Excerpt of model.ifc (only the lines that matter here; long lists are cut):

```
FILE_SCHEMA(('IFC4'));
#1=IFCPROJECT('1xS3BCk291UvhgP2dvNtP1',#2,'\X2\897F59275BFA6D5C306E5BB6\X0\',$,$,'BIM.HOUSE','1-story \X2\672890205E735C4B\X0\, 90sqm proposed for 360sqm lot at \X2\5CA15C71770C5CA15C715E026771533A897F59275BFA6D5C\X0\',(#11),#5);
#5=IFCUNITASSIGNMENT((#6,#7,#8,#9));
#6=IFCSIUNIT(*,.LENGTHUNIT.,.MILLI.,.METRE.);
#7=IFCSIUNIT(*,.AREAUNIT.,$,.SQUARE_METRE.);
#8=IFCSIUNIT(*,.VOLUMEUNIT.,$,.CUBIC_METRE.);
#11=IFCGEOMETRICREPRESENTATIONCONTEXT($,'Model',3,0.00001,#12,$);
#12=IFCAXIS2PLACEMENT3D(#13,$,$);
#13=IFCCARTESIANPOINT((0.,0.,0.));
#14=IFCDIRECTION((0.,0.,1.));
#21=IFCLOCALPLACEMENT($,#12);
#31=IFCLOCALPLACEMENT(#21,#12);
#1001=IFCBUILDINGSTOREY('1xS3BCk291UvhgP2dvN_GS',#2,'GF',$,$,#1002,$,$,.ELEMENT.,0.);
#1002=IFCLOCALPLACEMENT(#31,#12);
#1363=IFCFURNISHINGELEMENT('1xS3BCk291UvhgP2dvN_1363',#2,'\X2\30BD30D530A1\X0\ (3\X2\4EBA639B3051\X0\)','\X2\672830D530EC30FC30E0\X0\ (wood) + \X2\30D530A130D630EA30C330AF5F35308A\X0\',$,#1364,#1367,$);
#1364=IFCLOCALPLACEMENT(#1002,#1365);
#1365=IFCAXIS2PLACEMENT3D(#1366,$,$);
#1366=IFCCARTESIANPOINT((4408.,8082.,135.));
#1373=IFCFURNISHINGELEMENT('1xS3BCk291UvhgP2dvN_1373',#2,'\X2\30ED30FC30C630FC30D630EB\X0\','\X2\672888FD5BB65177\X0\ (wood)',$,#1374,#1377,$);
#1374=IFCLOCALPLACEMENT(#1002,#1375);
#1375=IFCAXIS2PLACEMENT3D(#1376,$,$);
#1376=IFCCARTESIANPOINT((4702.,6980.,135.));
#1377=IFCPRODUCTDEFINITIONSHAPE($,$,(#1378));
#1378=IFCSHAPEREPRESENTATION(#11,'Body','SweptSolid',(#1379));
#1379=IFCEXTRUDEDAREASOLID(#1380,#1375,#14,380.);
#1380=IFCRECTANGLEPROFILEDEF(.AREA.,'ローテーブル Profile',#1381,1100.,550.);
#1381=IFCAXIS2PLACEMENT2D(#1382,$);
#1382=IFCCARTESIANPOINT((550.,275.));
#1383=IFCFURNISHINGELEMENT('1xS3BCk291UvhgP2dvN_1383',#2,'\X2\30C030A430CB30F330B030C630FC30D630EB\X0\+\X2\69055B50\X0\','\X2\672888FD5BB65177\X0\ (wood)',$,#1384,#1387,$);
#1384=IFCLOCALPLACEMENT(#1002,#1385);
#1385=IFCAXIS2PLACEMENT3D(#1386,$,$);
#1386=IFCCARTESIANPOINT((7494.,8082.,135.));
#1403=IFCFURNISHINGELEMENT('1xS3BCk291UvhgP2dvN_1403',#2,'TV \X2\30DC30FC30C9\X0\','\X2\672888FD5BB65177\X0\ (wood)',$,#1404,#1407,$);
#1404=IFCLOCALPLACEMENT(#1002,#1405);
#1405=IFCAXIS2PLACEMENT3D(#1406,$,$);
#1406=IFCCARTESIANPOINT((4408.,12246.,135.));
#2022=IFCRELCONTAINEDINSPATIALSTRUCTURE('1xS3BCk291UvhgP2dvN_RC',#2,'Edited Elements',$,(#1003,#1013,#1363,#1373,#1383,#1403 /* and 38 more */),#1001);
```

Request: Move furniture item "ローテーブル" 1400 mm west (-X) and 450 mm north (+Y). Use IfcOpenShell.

```python
import ifcopenshell
import ifcopenshell.api.geometry
import ifcopenshell.util.placement

model = ifcopenshell.open("model.ifc")

item = model.by_id(1373)
matrix = ifcopenshell.util.placement.get_local_placement(item.ObjectPlacement)
matrix[0, 3] -= 1400.0
matrix[1, 3] += 450.0
ifcopenshell.api.geometry.edit_object_placement(model, product=item, matrix=matrix, is_si=False)

print(ifcopenshell.util.placement.get_local_placement(item.ObjectPlacement).round(3) + 0.0)

model.write("model-out.ifc")
```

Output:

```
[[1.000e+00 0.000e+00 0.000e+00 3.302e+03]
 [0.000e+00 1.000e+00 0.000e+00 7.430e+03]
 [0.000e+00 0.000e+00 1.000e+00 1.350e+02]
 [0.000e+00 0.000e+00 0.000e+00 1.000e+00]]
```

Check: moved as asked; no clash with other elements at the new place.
